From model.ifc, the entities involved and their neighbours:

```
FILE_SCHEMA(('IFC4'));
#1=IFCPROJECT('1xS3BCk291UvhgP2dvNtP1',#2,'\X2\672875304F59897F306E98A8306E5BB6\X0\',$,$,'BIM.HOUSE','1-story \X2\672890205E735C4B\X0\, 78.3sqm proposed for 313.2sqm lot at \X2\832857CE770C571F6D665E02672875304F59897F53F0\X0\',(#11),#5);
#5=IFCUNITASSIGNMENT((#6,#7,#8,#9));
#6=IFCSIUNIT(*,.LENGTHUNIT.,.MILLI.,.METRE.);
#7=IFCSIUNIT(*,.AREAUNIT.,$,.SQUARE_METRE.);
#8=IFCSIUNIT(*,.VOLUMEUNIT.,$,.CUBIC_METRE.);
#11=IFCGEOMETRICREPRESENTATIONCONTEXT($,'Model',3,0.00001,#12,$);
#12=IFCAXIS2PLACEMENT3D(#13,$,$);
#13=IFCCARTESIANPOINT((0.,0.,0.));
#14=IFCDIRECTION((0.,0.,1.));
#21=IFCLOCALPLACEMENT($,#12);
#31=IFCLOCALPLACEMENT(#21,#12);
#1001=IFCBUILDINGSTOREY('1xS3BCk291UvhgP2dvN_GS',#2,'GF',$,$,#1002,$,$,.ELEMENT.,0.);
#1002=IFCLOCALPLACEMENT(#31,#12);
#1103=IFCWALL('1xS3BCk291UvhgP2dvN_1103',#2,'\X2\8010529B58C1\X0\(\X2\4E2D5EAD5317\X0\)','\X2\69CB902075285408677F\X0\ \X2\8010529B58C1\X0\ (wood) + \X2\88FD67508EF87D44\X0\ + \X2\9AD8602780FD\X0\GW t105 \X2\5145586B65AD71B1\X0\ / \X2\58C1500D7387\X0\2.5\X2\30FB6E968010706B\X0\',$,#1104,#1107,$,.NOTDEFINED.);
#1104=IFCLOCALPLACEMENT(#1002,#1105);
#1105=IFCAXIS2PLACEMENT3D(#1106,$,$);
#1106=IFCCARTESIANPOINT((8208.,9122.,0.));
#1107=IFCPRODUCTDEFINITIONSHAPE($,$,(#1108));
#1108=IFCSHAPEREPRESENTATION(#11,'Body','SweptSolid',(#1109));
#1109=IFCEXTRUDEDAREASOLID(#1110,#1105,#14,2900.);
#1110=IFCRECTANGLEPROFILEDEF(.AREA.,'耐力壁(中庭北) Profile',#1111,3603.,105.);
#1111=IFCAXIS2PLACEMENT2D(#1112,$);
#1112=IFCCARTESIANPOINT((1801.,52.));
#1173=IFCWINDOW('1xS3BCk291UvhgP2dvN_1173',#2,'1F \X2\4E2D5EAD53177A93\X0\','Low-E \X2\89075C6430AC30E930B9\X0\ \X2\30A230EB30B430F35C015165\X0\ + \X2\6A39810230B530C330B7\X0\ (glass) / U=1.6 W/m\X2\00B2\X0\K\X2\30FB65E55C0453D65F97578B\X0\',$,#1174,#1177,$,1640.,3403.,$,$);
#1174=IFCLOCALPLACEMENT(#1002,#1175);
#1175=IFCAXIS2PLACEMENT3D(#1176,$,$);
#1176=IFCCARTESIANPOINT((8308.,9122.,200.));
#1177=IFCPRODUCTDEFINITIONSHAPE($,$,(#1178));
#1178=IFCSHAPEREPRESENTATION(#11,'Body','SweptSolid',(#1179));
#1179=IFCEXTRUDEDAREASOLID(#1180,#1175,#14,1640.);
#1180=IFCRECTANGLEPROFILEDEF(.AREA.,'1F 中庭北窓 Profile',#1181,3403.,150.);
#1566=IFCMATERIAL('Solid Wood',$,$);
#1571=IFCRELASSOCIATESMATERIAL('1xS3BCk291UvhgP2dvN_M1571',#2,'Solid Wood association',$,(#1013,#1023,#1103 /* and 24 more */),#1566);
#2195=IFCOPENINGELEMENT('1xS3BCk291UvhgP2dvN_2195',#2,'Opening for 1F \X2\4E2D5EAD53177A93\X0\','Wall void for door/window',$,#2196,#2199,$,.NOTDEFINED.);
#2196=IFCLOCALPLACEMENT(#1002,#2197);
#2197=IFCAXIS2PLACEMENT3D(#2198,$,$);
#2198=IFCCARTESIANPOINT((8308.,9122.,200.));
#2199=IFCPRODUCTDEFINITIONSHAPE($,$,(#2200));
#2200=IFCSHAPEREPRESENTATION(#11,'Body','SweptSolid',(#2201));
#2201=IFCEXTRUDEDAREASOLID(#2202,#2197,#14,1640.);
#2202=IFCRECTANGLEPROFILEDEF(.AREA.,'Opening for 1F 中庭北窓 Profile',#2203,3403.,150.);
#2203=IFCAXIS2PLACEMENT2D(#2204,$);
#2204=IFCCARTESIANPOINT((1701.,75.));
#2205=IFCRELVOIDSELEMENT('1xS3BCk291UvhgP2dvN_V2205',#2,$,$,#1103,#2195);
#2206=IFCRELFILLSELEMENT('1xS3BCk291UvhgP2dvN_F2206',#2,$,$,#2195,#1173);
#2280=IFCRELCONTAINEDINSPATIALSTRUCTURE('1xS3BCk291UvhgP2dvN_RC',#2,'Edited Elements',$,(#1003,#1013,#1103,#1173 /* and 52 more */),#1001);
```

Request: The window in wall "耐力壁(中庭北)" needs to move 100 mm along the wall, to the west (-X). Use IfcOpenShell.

```python
import ifcopenshell
import ifcopenshell.api.geometry
import ifcopenshell.util.placement
import ifcopenshell.util.unit

model = ifcopenshell.open("model.ifc")
unit_scale = ifcopenshell.util.unit.calculate_unit_scale(model)

window = model.by_guid("1xS3BCk291UvhgP2dvN_1173")
opening = window.FillsVoids[0].RelatingOpeningElement
wall = opening.VoidsElements[0].RelatingBuildingElement

wall_matrix = ifcopenshell.util.placement.get_local_placement(wall.ObjectPlacement)
shift = wall_matrix[:3, 0] * -0.1 / unit_scale
before = ifcopenshell.util.placement.get_local_placement(window.ObjectPlacement)[:3, 3].copy()

# The window is not placed relative to its opening, so move both.
for product in (opening, window):
    matrix = ifcopenshell.util.placement.get_local_placement(product.ObjectPlacement)
    matrix[:3, 3] += shift
    ifcopenshell.api.geometry.edit_object_placement(model, product=product, matrix=matrix, is_si=False)

after = ifcopenshell.util.placement.get_local_placement(window.ObjectPlacement)[:3, 3]
print("window moved by", (after - before).round(3) + 0.0)

model.write("model_v2.ifc")
```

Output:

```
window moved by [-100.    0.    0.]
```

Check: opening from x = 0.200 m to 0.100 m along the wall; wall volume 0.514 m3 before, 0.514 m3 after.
